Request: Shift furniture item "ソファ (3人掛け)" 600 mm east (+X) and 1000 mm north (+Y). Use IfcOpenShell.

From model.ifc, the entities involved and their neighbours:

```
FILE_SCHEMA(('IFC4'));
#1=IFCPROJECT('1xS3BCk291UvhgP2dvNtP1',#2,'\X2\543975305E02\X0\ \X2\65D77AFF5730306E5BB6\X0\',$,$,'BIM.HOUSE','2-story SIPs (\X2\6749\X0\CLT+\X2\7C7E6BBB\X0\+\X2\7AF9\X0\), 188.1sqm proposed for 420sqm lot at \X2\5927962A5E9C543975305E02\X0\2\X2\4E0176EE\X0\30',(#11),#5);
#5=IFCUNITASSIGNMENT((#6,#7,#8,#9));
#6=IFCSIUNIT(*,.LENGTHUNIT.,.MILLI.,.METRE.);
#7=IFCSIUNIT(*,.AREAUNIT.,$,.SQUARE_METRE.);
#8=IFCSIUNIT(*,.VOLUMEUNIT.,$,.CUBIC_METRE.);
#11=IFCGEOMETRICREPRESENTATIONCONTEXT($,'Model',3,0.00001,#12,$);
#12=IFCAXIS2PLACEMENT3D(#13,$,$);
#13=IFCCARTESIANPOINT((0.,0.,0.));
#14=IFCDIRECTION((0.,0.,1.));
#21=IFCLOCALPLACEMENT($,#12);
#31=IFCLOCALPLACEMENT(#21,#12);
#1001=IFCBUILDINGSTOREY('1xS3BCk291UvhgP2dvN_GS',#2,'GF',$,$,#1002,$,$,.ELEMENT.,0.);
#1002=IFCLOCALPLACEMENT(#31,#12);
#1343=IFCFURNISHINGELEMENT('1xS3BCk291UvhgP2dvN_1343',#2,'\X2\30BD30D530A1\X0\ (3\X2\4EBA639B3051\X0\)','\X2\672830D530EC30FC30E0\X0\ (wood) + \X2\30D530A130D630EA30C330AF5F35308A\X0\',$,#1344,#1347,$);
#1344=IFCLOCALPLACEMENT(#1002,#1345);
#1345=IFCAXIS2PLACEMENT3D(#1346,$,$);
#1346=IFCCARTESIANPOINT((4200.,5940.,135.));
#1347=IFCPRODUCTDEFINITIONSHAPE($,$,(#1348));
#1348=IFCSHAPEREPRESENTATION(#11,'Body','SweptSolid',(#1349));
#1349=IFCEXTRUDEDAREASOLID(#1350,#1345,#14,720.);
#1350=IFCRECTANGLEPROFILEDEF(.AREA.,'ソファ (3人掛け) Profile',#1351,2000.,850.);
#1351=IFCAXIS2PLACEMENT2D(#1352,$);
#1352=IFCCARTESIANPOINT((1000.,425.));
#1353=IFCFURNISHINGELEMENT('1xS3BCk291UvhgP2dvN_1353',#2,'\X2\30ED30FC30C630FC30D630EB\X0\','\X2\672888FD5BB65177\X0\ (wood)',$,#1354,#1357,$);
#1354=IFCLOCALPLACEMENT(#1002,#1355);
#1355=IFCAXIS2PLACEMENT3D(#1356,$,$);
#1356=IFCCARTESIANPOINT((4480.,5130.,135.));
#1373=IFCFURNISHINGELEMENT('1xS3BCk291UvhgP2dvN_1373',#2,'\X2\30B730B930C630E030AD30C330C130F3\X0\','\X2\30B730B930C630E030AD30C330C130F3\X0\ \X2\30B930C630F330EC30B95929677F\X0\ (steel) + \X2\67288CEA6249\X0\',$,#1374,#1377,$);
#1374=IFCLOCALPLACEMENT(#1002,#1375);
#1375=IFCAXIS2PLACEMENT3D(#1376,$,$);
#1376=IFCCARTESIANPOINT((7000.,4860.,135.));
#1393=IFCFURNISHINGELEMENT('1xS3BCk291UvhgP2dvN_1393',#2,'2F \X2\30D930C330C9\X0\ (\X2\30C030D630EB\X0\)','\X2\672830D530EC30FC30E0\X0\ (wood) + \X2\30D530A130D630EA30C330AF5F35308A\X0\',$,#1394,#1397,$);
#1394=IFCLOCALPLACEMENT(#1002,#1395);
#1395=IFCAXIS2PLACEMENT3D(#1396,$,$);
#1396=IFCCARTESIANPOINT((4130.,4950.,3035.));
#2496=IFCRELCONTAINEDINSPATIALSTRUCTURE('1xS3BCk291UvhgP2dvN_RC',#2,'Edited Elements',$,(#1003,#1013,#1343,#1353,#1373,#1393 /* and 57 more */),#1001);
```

```python
import ifcopenshell
import ifcopenshell.api.geometry
import ifcopenshell.util.placement
import ifcopenshell.util.unit

model = ifcopenshell.open("model.ifc")
unit_scale = ifcopenshell.util.unit.calculate_unit_scale(model)

item = model.by_guid("1xS3BCk291UvhgP2dvN_1343")
matrix = ifcopenshell.util.placement.get_local_placement(item.ObjectPlacement)
matrix[0, 3] += 0.6 / unit_scale
matrix[1, 3] += 1 / unit_scale
ifcopenshell.api.geometry.edit_object_placement(model, product=item, matrix=matrix, is_si=False)

print(ifcopenshell.util.placement.get_local_placement(item.ObjectPlacement).round(3) + 0.0)

model.write("model-out.ifc")
```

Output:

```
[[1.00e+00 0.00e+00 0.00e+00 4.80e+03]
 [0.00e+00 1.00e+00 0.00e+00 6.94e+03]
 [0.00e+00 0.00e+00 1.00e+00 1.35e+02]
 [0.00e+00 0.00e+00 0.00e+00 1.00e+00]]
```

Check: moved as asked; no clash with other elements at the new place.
